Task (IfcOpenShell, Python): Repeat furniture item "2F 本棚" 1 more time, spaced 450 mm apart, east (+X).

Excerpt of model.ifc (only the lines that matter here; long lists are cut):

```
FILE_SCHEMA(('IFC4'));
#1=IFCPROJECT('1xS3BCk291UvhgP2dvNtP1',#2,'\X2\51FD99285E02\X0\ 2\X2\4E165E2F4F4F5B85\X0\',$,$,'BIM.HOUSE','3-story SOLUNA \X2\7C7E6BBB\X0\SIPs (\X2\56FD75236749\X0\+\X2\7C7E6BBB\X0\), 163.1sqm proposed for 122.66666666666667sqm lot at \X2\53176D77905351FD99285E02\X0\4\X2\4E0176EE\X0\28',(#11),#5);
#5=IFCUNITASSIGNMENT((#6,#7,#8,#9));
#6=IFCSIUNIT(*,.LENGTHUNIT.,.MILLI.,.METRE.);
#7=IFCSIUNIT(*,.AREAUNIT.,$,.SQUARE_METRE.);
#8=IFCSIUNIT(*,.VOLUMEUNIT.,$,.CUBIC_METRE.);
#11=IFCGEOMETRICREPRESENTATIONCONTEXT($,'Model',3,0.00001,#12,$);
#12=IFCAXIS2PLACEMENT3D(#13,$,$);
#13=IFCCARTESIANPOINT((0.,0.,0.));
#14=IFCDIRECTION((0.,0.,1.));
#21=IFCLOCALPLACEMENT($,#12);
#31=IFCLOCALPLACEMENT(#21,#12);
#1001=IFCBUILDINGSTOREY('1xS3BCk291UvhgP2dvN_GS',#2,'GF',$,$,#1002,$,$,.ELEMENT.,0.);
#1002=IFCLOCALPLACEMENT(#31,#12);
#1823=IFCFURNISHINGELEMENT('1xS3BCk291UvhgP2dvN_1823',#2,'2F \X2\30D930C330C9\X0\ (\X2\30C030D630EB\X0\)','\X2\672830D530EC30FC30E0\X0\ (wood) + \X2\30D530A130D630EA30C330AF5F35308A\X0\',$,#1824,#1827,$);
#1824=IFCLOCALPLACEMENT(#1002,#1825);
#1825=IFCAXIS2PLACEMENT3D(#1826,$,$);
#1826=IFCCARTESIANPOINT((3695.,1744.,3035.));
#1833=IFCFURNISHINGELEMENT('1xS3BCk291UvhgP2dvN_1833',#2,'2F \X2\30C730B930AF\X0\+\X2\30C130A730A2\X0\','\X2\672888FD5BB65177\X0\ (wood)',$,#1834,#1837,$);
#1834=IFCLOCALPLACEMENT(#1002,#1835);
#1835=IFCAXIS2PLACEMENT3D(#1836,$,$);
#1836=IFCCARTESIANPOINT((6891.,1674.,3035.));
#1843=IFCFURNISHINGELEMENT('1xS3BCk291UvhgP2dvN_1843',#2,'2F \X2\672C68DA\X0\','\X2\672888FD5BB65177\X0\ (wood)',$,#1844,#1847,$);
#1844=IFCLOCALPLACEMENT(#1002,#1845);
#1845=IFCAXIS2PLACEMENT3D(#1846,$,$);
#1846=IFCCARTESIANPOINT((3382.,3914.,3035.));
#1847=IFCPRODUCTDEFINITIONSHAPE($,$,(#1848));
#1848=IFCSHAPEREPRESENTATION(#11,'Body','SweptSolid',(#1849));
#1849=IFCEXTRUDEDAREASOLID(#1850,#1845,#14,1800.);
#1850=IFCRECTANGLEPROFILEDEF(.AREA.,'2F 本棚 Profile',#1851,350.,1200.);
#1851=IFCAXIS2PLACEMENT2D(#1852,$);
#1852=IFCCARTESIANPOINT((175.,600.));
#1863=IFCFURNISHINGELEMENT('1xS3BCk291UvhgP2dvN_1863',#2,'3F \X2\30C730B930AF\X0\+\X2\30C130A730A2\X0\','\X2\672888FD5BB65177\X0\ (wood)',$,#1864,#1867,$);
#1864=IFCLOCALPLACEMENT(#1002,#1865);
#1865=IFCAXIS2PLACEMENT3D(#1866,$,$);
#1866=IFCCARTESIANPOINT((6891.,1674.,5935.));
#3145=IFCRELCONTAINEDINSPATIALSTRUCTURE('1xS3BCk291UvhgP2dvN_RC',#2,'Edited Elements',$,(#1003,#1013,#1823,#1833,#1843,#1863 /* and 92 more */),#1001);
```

```python
import numpy as np
import ifcopenshell
import ifcopenshell.api.geometry
import ifcopenshell.api.root
import ifcopenshell.util.element
import ifcopenshell.util.placement
import ifcopenshell.util.unit

model = ifcopenshell.open("model.ifc")
unit_scale = ifcopenshell.util.unit.calculate_unit_scale(model)


def reuse_history(source, copy):
    """copy_class also copies each property set's owner history, people and application; keep the originals."""
    for rel in copy.IsDefinedBy:
        if rel.is_a("IfcRelDefinesByProperties") and (history := rel.RelatingPropertyDefinition.OwnerHistory):
            rel.RelatingPropertyDefinition.OwnerHistory = source.OwnerHistory
            ifcopenshell.util.element.remove_deep2(model, history)


source = model.by_guid("1xS3BCk291UvhgP2dvN_1843")
base = ifcopenshell.util.placement.get_local_placement(source.ObjectPlacement)
step = np.array([1.0, 0.0, 0.0]) * 0.45 / unit_scale

for i in range(1, 2):
    copy = ifcopenshell.api.root.copy_class(model, product=source)
    copy.Representation = ifcopenshell.util.element.copy_deep(
        model, source.Representation, exclude=["IfcGeometricRepresentationContext", "IfcRepresentationMap"]
    )
    reuse_history(source, copy)
    matrix = base.copy()
    matrix[:3, 3] += i * step
    print("added at", matrix[:3, 3].round(3) + 0.0)
    ifcopenshell.api.geometry.edit_object_placement(model, product=copy, matrix=matrix, is_si=False)

model.write("model_v2.ifc")
```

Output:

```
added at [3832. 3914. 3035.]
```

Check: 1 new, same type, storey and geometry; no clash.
